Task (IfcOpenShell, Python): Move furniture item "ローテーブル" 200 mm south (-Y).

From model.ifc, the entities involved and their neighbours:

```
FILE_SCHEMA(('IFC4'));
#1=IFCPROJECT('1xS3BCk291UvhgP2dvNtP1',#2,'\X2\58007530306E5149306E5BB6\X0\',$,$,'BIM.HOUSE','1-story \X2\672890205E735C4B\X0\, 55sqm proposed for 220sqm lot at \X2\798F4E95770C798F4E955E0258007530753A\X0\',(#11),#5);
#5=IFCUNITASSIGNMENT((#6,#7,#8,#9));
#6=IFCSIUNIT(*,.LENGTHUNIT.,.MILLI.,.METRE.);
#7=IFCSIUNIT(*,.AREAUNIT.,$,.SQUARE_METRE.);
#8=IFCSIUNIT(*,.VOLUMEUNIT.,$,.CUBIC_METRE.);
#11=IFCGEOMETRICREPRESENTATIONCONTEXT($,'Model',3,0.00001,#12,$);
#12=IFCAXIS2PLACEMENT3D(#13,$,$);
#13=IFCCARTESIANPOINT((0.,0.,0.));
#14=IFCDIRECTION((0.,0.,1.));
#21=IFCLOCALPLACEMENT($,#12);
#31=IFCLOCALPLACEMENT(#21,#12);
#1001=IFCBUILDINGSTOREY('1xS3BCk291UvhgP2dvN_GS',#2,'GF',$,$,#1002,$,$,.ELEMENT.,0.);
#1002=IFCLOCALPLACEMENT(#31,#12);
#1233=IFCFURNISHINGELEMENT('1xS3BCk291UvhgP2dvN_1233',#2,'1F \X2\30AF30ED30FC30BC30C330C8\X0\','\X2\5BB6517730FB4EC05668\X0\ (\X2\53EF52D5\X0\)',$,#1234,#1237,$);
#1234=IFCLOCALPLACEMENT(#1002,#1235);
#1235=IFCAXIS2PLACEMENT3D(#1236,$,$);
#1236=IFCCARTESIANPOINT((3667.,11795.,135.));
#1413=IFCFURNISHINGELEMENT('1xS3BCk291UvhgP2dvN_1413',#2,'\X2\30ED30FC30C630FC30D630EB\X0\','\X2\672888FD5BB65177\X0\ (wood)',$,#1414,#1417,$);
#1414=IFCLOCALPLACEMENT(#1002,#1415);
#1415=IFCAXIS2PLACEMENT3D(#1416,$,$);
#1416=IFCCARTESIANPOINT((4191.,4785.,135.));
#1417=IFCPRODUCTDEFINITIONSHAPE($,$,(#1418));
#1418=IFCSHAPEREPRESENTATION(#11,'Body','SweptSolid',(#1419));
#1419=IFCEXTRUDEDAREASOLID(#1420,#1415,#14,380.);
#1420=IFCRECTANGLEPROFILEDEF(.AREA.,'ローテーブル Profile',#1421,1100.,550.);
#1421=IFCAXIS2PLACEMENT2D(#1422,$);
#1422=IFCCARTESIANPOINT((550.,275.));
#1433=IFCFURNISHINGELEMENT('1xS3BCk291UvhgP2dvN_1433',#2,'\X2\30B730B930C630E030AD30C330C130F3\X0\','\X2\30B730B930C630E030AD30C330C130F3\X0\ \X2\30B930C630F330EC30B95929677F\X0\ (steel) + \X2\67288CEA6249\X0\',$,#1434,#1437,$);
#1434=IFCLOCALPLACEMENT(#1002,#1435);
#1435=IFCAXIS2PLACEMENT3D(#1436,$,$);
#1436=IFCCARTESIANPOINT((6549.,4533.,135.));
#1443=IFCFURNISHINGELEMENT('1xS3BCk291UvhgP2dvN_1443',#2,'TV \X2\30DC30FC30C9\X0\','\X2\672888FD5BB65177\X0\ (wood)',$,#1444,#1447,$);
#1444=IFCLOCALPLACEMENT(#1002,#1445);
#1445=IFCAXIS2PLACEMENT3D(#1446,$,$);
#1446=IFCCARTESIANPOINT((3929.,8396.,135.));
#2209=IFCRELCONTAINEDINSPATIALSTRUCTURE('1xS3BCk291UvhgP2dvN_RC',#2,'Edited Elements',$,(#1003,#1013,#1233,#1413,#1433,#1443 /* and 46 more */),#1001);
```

```python
import ifcopenshell
import ifcopenshell.api.geometry
import ifcopenshell.util.placement
import ifcopenshell.util.unit

model = ifcopenshell.open("model.ifc")
unit_scale = ifcopenshell.util.unit.calculate_unit_scale(model)

item = model.by_guid("1xS3BCk291UvhgP2dvN_1413")
matrix = ifcopenshell.util.placement.get_local_placement(item.ObjectPlacement)
matrix[1, 3] -= 0.2 / unit_scale
ifcopenshell.api.geometry.edit_object_placement(model, product=item, matrix=matrix, is_si=False)

print(ifcopenshell.util.placement.get_local_placement(item.ObjectPlacement).round(3) + 0.0)

model.write("model_rev.ifc")
```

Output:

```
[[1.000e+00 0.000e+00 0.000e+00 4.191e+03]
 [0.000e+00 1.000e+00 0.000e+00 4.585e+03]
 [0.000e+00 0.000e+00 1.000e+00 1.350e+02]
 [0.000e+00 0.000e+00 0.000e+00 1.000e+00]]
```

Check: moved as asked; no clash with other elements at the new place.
